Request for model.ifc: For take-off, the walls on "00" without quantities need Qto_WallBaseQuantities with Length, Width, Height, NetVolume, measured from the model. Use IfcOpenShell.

First a look at what the model holds.

```python
import ifcopenshell
import ifcopenshell.util.element
import ifcopenshell.util.unit

model = ifcopenshell.open("model.ifc")
print(model.schema)
for unit_type in ("LENGTHUNIT", "AREAUNIT", "VOLUMEUNIT"):
    print(unit_type, ifcopenshell.util.unit.calculate_unit_scale(model, unit_type))
storey = next(s for s in model.by_type("IfcBuildingStorey") if s.Name == "00")
walls = [e for e in ifcopenshell.util.element.get_decomposition(storey) if e.is_a("IfcWall")]
for e in sorted(walls, key=lambda e: e.id()):
    print(e.id(), e.is_a(), e.Name, list(ifcopenshell.util.element.get_psets(e, qtos_only=True)), sep=" | ")
```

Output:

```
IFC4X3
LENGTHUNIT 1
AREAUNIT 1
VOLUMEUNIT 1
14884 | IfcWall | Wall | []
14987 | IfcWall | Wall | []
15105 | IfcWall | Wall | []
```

```python
import ifcopenshell
import ifcopenshell.api.pset
import ifcopenshell.geom
import ifcopenshell.util.element
import ifcopenshell.util.shape
import ifcopenshell.util.unit

model = ifcopenshell.open("model.ifc")
unit_scale = ifcopenshell.util.unit.calculate_unit_scale(model)
volume_scale = ifcopenshell.util.unit.calculate_unit_scale(model, "VOLUMEUNIT")
settings = ifcopenshell.geom.settings()

storey = next(s for s in model.by_type("IfcBuildingStorey") if s.Name == "00")
walls = [e for e in ifcopenshell.util.element.get_decomposition(storey) if e.is_a("IfcWall")]

for e in sorted(walls, key=lambda e: e.id()):
    if ifcopenshell.util.element.get_psets(e, qtos_only=True, should_inherit=False):
        continue
    # Geometry comes back in metres, in the element's own axes.
    shape = ifcopenshell.geom.create_shape(settings, e)
    values = {
        "Length": ifcopenshell.util.shape.get_x(shape.geometry) / unit_scale,
        "Width": ifcopenshell.util.shape.get_y(shape.geometry) / unit_scale,
        "Height": ifcopenshell.util.shape.get_z(shape.geometry) / unit_scale,
        "NetVolume": ifcopenshell.util.shape.get_volume(shape.geometry) / volume_scale,
    }
    qto = ifcopenshell.api.pset.add_qto(model, product=e, name="Qto_WallBaseQuantities")
    ifcopenshell.api.pset.edit_qto(model, qto=qto, properties=values)
    print(e.id(), {k: round(v, 3) for k, v in values.items()})

model.write("model_edited.ifc")
```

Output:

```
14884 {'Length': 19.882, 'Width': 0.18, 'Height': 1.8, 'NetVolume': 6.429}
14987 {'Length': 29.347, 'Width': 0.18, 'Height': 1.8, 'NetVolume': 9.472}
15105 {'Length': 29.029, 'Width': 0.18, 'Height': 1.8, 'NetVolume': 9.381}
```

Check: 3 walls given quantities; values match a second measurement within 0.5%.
